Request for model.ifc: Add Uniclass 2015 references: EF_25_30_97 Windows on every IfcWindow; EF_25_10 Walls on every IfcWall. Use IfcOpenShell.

First a look at what the model holds.

```python
import ifcopenshell

model = ifcopenshell.open("model.ifc")
print(model.schema)
print("classifications:", [c.Name for c in model.by_type("IfcClassification")])
for ifc_class in ("IfcDoor", "IfcRoof", "IfcStair", "IfcWall", "IfcWindow"):
    print(ifc_class, len(model.by_type(ifc_class)))
```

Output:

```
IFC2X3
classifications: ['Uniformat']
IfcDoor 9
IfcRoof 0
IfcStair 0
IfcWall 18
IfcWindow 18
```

```python
import ifcopenshell
import ifcopenshell.api.classification

model = ifcopenshell.open("model.ifc")

# IFC2X3 requires Source and Edition and has no link from the project to the system.
system = model.create_entity("IfcClassification", Source="NBS", Edition="2015", Name="Uniclass 2015")

codes = {
    "IfcWindow": ("EF_25_30_97", "Windows"),
    "IfcWall": ("EF_25_10", "Walls"),
}
for ifc_class, (code, name) in codes.items():
    products = model.by_type(ifc_class)
    ifcopenshell.api.classification.add_reference(
        model, products=products, classification=system, identification=code, name=name
    )
    print(code, len(products))

model.write("model_updated.ifc")
```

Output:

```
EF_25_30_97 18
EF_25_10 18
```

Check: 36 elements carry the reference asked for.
